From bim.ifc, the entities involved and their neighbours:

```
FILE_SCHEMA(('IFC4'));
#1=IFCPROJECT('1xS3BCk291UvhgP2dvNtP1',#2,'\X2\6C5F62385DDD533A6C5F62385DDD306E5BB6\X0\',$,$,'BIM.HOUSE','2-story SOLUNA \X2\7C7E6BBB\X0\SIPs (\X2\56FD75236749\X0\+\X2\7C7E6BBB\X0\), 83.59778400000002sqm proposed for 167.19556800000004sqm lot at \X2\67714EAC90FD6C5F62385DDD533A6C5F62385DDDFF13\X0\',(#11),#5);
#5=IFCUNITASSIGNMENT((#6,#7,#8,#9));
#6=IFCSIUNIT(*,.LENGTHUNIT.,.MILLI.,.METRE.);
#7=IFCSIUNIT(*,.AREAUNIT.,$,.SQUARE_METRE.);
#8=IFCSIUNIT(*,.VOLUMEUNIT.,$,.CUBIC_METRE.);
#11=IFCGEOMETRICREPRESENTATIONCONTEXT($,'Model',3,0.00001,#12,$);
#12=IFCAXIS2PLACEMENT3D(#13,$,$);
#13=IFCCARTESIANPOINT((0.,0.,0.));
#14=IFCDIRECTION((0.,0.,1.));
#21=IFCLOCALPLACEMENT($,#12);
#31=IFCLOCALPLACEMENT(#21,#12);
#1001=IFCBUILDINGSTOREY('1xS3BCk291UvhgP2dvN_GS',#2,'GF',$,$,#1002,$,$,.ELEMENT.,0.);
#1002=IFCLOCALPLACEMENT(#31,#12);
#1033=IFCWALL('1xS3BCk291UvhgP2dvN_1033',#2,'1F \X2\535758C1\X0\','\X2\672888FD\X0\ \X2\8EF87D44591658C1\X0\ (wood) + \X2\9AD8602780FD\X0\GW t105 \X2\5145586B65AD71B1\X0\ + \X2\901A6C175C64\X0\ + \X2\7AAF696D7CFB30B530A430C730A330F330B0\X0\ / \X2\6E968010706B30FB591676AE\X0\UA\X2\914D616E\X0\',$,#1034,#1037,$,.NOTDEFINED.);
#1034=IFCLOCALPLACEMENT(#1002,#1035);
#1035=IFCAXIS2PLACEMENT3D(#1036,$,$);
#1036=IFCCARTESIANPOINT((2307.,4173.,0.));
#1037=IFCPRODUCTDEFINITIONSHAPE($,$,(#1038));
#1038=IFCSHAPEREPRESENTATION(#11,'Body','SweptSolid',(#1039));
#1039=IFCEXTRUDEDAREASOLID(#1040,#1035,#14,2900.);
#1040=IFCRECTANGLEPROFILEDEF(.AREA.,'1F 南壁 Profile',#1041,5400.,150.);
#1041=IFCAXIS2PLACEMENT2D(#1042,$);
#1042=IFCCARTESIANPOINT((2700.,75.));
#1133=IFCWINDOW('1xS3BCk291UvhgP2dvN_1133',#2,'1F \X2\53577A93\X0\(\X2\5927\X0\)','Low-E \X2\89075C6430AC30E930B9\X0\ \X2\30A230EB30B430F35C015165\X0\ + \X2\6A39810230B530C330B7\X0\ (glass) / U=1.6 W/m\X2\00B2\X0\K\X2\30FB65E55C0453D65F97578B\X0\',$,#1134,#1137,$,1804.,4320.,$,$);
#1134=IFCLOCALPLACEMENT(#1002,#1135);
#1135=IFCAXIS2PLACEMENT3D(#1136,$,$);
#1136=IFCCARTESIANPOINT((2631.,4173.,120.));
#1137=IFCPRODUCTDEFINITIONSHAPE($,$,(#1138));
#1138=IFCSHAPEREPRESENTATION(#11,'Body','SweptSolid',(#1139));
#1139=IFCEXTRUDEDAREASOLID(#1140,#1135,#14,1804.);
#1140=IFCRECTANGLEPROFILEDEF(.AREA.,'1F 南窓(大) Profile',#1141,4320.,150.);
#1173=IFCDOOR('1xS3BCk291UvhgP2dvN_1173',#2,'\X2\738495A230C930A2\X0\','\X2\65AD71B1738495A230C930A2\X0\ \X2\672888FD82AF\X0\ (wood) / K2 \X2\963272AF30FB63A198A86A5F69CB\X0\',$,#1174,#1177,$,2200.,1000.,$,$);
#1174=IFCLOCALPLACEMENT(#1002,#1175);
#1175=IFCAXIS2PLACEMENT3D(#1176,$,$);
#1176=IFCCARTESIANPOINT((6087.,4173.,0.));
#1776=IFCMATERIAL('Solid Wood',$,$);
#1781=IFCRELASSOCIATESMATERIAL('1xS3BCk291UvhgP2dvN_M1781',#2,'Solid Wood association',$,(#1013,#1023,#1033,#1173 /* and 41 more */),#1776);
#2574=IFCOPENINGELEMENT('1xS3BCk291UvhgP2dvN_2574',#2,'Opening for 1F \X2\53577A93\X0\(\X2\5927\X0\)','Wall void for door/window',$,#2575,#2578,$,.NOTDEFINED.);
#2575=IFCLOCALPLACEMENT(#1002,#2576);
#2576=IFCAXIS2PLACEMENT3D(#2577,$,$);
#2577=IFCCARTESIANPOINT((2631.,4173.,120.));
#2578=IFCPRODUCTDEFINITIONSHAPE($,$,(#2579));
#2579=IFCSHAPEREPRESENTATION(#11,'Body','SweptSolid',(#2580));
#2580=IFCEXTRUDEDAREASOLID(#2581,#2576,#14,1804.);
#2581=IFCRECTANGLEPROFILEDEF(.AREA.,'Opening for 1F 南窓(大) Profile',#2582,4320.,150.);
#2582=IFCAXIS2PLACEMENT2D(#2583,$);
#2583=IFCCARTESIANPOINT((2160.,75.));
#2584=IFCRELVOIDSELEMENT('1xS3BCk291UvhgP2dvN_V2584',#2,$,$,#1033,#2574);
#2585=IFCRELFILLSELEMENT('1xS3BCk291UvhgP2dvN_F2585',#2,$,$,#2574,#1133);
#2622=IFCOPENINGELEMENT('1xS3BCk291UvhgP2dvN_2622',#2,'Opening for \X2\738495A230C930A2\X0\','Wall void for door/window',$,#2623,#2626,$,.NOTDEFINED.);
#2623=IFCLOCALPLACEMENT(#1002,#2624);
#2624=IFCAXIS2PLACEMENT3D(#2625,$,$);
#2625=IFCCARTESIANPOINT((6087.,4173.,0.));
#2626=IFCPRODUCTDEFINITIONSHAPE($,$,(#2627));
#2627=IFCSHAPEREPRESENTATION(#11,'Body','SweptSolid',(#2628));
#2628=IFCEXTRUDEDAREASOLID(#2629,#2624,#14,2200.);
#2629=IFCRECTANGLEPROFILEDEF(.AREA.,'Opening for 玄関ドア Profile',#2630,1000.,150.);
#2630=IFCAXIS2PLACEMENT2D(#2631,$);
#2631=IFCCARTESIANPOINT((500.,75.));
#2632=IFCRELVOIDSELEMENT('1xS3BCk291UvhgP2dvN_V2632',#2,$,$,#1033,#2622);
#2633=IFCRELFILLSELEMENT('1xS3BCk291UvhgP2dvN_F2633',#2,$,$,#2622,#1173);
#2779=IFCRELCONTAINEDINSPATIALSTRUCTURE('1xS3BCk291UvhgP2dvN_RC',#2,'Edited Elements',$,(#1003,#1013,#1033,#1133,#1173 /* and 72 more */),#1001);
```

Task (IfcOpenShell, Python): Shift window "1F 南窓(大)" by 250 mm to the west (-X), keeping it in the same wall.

```python
import ifcopenshell
import ifcopenshell.api.geometry
import ifcopenshell.util.placement
import ifcopenshell.util.unit

model = ifcopenshell.open("bim.ifc")
unit_scale = ifcopenshell.util.unit.calculate_unit_scale(model)

window = model.by_guid("1xS3BCk291UvhgP2dvN_1133")
opening = window.FillsVoids[0].RelatingOpeningElement
wall = opening.VoidsElements[0].RelatingBuildingElement

wall_matrix = ifcopenshell.util.placement.get_local_placement(wall.ObjectPlacement)
shift = wall_matrix[:3, 0] * -0.25 / unit_scale
before = ifcopenshell.util.placement.get_local_placement(window.ObjectPlacement)[:3, 3].copy()

# The window is not placed relative to its opening, so move both.
for product in (opening, window):
    matrix = ifcopenshell.util.placement.get_local_placement(product.ObjectPlacement)
    matrix[:3, 3] += shift
    ifcopenshell.api.geometry.edit_object_placement(model, product=product, matrix=matrix, is_si=False)

after = ifcopenshell.util.placement.get_local_placement(window.ObjectPlacement)[:3, 3]
print("window moved by", (after - before).round(3) + 0.0)

model.write("bim-out.ifc")
```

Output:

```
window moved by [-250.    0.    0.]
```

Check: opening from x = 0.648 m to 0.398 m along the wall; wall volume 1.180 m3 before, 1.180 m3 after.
